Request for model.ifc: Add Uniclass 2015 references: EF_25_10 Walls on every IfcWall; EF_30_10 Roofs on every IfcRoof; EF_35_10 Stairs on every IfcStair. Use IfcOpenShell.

First a look at what the model holds.

```python
import ifcopenshell

model = ifcopenshell.open("model.ifc")
print(model.schema)
print("classifications:", [c.Name for c in model.by_type("IfcClassification")])
for ifc_class in ("IfcDoor", "IfcRoof", "IfcStair", "IfcWall", "IfcWindow"):
    print(ifc_class, len(model.by_type(ifc_class)))
```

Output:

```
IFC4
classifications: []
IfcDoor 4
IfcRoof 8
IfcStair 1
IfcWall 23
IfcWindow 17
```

```python
import ifcopenshell
import ifcopenshell.api.classification

model = ifcopenshell.open("model.ifc")

system = ifcopenshell.api.classification.add_classification(model, classification="Uniclass 2015")

codes = {
    "IfcWall": ("EF_25_10", "Walls"),
    "IfcRoof": ("EF_30_10", "Roofs"),
    "IfcStair": ("EF_35_10", "Stairs"),
}
for ifc_class, (code, name) in codes.items():
    products = model.by_type(ifc_class)
    ifcopenshell.api.classification.add_reference(
        model, products=products, classification=system, identification=code, name=name
    )
    print(code, len(products))

model.write("model_updated.ifc")
```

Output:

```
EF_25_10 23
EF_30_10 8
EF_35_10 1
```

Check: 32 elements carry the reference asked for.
